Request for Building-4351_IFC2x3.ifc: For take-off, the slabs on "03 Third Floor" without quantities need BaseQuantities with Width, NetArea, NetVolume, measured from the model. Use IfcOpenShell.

First a look at what the model holds.

```python
import ifcopenshell
import ifcopenshell.util.element
import ifcopenshell.util.unit

model = ifcopenshell.open("Building-4351_IFC2x3.ifc")
print(model.schema)
for unit_type in ("LENGTHUNIT", "AREAUNIT", "VOLUMEUNIT"):
    print(unit_type, ifcopenshell.util.unit.calculate_unit_scale(model, unit_type))
storey = next(s for s in model.by_type("IfcBuildingStorey") if s.Name == "03 Third Floor")
slabs = [e for e in ifcopenshell.util.element.get_decomposition(storey) if e.is_a("IfcSlab")]
for e in sorted(slabs, key=lambda e: e.id()):
    print(e.id(), e.is_a(), e.Name, list(ifcopenshell.util.element.get_psets(e, qtos_only=True)), sep=" | ")
```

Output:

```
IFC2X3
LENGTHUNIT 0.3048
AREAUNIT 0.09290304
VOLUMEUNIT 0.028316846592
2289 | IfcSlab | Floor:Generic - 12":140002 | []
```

```python
import ifcopenshell
import ifcopenshell.api.pset
import ifcopenshell.geom
import ifcopenshell.util.element
import ifcopenshell.util.shape
import ifcopenshell.util.unit

model = ifcopenshell.open("Building-4351_IFC2x3.ifc")
unit_scale = ifcopenshell.util.unit.calculate_unit_scale(model)
area_scale = ifcopenshell.util.unit.calculate_unit_scale(model, "AREAUNIT")
volume_scale = ifcopenshell.util.unit.calculate_unit_scale(model, "VOLUMEUNIT")
settings = ifcopenshell.geom.settings()

storey = next(s for s in model.by_type("IfcBuildingStorey") if s.Name == "03 Third Floor")
slabs = [e for e in ifcopenshell.util.element.get_decomposition(storey) if e.is_a("IfcSlab")]

for e in sorted(slabs, key=lambda e: e.id()):
    if ifcopenshell.util.element.get_psets(e, qtos_only=True, should_inherit=False):
        continue
    # Geometry comes back in metres, in the element's own axes.
    shape = ifcopenshell.geom.create_shape(settings, e)
    values = {
        "Width": ifcopenshell.util.shape.get_z(shape.geometry) / unit_scale,
        "NetArea": ifcopenshell.util.shape.get_footprint_area(shape.geometry) / area_scale,
        "NetVolume": ifcopenshell.util.shape.get_volume(shape.geometry) / volume_scale,
    }
    qto = ifcopenshell.api.pset.add_qto(model, product=e, name="BaseQuantities")
    ifcopenshell.api.pset.edit_qto(model, qto=qto, properties=values)
    print(e.id(), {k: round(v, 3) for k, v in values.items()})

model.write("Building-4351_IFC2x3-out.ifc")
```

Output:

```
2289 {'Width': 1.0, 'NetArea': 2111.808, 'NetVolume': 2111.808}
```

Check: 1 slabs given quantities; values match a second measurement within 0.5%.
